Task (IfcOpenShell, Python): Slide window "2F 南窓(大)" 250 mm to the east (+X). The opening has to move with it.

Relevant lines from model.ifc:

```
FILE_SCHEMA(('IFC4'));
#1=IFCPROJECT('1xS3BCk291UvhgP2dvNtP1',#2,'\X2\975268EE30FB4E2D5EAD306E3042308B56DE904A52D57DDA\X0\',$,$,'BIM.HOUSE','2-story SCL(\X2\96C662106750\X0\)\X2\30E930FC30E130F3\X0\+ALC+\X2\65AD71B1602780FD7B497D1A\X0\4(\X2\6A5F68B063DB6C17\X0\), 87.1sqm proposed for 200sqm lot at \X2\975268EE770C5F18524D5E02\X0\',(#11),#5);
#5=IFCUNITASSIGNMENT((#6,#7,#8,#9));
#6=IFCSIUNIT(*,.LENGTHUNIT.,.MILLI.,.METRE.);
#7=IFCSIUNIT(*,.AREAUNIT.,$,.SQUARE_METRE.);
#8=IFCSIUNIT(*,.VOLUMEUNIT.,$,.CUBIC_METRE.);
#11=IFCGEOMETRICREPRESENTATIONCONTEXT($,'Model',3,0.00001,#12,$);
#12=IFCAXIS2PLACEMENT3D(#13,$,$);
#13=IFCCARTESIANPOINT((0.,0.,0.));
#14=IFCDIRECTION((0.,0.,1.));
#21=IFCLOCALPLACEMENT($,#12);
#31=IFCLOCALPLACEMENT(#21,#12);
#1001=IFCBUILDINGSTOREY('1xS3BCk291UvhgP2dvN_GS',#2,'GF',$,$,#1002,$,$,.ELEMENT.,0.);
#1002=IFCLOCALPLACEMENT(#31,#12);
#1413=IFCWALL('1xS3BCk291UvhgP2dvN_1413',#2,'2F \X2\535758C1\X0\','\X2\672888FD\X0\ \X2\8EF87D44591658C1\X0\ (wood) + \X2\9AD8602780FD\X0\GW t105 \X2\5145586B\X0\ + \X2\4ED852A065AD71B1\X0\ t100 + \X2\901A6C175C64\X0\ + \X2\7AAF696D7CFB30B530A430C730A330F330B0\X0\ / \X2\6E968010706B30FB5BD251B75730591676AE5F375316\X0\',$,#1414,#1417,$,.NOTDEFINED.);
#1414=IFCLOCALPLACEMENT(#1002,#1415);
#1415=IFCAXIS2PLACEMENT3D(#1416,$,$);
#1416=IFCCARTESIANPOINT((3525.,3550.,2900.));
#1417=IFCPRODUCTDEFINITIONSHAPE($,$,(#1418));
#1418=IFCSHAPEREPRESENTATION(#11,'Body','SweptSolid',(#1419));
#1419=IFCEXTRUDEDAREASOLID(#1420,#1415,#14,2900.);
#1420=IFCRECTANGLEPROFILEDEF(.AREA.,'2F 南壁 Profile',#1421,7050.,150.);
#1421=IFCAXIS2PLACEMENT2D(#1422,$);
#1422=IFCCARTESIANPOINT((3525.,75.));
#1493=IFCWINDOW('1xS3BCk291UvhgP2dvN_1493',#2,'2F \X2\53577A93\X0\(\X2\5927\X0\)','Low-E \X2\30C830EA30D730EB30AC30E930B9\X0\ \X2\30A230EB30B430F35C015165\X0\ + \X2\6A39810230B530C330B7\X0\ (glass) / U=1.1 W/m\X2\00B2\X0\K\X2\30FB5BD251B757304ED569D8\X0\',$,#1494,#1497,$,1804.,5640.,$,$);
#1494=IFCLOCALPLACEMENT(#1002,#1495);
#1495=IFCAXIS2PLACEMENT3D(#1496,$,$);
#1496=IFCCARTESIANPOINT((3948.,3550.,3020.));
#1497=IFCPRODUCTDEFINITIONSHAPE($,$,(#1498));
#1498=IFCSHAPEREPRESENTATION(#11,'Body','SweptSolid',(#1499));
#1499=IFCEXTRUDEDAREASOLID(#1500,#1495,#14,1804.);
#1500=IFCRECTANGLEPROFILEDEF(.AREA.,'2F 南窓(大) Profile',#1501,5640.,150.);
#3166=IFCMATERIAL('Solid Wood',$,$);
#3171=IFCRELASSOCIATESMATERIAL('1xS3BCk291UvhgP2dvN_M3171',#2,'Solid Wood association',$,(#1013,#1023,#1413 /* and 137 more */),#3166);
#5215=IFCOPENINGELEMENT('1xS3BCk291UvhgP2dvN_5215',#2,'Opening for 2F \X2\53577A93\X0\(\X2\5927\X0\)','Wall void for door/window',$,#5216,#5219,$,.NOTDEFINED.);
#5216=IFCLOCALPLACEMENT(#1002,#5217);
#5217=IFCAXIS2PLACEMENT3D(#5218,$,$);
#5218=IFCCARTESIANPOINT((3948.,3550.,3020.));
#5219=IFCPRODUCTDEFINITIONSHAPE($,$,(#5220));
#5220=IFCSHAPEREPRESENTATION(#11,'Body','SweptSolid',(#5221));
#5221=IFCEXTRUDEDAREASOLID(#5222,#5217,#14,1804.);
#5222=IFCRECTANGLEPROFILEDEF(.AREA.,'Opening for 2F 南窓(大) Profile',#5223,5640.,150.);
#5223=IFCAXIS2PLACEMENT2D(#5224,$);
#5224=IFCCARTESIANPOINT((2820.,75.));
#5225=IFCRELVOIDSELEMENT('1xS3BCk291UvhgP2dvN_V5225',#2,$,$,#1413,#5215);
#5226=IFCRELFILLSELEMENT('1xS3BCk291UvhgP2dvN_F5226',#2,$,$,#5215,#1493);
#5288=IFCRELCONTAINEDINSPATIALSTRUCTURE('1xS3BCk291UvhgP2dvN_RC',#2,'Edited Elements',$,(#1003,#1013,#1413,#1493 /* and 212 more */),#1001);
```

```python
import ifcopenshell
import ifcopenshell.api.geometry
import ifcopenshell.util.placement

model = ifcopenshell.open("model.ifc")

window = model.by_guid("1xS3BCk291UvhgP2dvN_1493")
opening = window.FillsVoids[0].RelatingOpeningElement
wall = opening.VoidsElements[0].RelatingBuildingElement

wall_matrix = ifcopenshell.util.placement.get_local_placement(wall.ObjectPlacement)
shift = wall_matrix[:3, 0] * 250.0
before = ifcopenshell.util.placement.get_local_placement(window.ObjectPlacement)[:3, 3].copy()

# The window is not placed relative to its opening, so move both.
for product in (opening, window):
    matrix = ifcopenshell.util.placement.get_local_placement(product.ObjectPlacement)
    matrix[:3, 3] += shift
    ifcopenshell.api.geometry.edit_object_placement(model, product=product, matrix=matrix, is_si=False)

after = ifcopenshell.util.placement.get_local_placement(window.ObjectPlacement)[:3, 3]
print("window moved by", (after - before).round(3) + 0.0)

model.write("model_edited.ifc")
```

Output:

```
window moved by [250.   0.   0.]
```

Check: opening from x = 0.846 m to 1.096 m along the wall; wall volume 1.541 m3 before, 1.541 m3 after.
